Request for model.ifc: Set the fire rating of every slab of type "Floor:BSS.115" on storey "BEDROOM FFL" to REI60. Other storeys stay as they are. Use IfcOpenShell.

First a look at what the model holds.

```python
import ifcopenshell
import ifcopenshell.util.element

model = ifcopenshell.open("model.ifc")
print(model.schema)
storey = next(s for s in model.by_type("IfcBuildingStorey") if s.Name == "BEDROOM FFL")
slabs = [e for e in ifcopenshell.util.element.get_decomposition(storey) if e.is_a("IfcSlab")]
seen = {}
for e in slabs:
    element_type = ifcopenshell.util.element.get_type(e)
    key = (element_type.Name if element_type != e and element_type else None, ifcopenshell.util.element.get_pset(e, "Pset_SlabCommon", "FireRating"))
    seen[key] = seen.get(key, 0) + 1
for (name, value), count in sorted(seen.items(), key=str):
    print(count, "x", name, "|", value)
```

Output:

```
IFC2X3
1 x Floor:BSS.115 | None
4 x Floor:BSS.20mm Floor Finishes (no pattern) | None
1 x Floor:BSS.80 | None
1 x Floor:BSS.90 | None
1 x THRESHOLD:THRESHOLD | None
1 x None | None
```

```python
import ifcopenshell
import ifcopenshell.api.pset
import ifcopenshell.util.element

model = ifcopenshell.open("model.ifc")

storey = next(s for s in model.by_type("IfcBuildingStorey") if s.Name == "BEDROOM FFL")
slabs = [e for e in ifcopenshell.util.element.get_decomposition(storey) if e.is_a("IfcSlab")]

count = 0
for e in slabs:
    element_type = ifcopenshell.util.element.get_type(e)
    if element_type in (None, e) or element_type.Name != "Floor:BSS.115":
        continue
    # add_pset returns the element's existing set when there is one.
    pset = ifcopenshell.api.pset.add_pset(model, product=e, name="Pset_SlabCommon")
    ifcopenshell.api.pset.edit_pset(model, pset=pset, properties={"FireRating": "REI60"})
    count += 1

print(count, "slabs updated")

model.write("model-out.ifc")
```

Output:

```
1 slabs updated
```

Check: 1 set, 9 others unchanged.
